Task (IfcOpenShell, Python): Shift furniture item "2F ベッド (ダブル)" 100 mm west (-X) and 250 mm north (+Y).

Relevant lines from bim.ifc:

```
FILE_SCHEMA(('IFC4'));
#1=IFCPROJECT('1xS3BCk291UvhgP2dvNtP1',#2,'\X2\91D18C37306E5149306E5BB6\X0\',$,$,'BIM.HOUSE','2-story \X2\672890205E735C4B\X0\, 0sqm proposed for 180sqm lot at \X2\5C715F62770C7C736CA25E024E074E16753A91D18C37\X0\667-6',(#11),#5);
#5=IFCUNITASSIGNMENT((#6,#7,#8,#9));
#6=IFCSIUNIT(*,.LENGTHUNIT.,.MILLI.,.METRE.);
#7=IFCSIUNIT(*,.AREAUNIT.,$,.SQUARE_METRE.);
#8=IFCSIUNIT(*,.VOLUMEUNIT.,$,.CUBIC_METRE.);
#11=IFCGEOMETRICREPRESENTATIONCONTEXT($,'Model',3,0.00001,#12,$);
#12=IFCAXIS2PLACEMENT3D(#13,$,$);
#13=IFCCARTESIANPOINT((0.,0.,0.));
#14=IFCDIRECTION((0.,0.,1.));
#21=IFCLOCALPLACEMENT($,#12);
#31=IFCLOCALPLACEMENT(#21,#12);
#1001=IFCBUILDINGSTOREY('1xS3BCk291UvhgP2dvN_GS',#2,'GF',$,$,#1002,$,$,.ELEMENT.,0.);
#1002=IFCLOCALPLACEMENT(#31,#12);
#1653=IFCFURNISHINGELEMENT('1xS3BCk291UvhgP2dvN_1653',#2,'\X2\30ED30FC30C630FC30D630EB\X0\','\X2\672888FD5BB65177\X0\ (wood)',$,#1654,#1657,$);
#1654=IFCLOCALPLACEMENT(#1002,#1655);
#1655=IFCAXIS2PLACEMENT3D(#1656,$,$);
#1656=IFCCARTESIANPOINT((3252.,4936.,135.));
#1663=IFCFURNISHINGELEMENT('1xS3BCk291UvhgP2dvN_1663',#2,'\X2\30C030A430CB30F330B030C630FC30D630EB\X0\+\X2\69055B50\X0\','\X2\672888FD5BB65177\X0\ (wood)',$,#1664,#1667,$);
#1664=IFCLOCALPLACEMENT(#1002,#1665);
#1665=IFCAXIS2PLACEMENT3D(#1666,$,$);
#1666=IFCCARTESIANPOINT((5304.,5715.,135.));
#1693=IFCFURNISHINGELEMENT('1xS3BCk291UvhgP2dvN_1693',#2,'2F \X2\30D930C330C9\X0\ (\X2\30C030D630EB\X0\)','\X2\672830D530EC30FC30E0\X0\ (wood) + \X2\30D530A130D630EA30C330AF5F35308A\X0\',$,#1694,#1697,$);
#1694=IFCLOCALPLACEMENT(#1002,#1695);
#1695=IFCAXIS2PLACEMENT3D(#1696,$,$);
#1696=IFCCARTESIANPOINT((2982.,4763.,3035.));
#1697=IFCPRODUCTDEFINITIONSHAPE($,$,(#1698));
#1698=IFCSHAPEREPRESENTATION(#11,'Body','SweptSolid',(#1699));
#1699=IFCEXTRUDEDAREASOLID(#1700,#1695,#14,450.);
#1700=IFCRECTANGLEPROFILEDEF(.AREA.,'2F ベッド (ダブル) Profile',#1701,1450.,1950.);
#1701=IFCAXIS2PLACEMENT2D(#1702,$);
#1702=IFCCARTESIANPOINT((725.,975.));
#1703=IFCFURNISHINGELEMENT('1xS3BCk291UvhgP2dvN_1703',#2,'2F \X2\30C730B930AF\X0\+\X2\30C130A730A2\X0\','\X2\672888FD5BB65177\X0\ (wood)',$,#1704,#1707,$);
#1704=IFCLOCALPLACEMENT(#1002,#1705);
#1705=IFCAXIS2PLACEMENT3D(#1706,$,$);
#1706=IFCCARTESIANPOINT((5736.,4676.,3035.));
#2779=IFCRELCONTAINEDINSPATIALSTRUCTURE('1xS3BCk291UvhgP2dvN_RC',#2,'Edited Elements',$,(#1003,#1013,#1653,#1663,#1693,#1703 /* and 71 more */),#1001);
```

```python
import ifcopenshell
import ifcopenshell.api.geometry
import ifcopenshell.util.placement
import ifcopenshell.util.unit

model = ifcopenshell.open("bim.ifc")
unit_scale = ifcopenshell.util.unit.calculate_unit_scale(model)

item = model.by_guid("1xS3BCk291UvhgP2dvN_1693")
matrix = ifcopenshell.util.placement.get_local_placement(item.ObjectPlacement)
matrix[0, 3] -= 0.1 / unit_scale
matrix[1, 3] += 0.25 / unit_scale
ifcopenshell.api.geometry.edit_object_placement(model, product=item, matrix=matrix, is_si=False)

print(ifcopenshell.util.placement.get_local_placement(item.ObjectPlacement).round(3) + 0.0)

model.write("bim_v2.ifc")
```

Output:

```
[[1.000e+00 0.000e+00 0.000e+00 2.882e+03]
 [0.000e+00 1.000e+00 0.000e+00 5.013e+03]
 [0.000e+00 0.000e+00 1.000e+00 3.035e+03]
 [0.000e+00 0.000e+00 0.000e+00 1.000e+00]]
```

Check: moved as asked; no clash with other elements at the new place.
